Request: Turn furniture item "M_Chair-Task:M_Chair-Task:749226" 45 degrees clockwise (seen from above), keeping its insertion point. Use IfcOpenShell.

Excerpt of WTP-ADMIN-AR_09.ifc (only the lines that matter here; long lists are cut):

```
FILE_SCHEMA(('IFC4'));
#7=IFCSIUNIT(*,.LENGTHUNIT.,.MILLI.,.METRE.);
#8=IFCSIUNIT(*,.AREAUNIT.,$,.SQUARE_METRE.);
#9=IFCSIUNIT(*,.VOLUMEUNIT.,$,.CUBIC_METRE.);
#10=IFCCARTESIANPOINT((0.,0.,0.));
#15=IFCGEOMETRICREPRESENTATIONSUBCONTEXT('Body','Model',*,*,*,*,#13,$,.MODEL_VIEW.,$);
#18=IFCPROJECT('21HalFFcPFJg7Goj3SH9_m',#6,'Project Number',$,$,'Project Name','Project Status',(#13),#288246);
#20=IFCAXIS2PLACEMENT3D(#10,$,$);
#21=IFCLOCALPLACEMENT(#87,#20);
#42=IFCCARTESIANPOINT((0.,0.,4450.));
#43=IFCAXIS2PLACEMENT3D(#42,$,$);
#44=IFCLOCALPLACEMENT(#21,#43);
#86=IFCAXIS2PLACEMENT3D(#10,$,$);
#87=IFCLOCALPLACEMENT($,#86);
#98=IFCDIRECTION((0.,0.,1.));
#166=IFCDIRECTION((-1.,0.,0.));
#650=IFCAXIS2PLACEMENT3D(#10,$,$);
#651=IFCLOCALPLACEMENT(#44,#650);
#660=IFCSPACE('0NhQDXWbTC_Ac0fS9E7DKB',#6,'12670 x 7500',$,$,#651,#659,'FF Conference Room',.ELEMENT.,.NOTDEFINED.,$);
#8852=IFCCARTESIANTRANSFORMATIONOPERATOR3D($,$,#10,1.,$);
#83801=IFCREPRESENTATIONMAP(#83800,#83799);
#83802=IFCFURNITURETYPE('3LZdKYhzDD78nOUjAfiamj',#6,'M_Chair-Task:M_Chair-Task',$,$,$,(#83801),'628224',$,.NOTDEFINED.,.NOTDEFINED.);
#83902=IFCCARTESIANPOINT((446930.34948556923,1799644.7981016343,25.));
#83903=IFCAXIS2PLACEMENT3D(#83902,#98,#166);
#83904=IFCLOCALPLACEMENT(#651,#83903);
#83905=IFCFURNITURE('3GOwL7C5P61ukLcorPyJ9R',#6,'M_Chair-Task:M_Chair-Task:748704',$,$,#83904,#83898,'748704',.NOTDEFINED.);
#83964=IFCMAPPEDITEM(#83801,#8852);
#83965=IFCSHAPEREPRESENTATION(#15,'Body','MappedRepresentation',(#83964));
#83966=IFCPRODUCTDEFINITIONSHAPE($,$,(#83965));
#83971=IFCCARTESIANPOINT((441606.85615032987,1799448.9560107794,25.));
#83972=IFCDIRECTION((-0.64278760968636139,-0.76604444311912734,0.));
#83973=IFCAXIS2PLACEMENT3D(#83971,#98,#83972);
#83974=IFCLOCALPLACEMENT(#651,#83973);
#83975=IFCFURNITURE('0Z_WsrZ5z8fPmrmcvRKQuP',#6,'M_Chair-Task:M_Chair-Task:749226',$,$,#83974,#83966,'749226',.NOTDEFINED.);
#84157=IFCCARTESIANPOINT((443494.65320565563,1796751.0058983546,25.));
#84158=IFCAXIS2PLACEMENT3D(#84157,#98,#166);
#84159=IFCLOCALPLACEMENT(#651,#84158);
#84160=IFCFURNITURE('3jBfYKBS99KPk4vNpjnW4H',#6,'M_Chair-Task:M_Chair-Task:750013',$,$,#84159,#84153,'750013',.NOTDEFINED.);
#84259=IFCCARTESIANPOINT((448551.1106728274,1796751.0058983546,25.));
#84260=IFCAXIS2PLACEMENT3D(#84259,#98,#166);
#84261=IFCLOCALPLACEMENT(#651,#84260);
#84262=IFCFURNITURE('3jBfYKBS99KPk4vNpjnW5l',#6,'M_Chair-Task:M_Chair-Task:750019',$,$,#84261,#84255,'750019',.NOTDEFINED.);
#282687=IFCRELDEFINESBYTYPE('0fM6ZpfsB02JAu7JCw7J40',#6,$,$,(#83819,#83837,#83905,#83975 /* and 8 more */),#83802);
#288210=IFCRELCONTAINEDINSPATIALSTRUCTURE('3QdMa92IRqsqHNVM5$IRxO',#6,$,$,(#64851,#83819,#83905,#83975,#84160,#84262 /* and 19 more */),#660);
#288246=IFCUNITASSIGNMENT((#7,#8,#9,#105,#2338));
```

```python
import ifcopenshell
import ifcopenshell.api.geometry
import ifcopenshell.util.placement

model = ifcopenshell.open("WTP-ADMIN-AR_09.ifc")

item = model.by_guid("0Z_WsrZ5z8fPmrmcvRKQuP")
matrix = ifcopenshell.util.placement.get_local_placement(item.ObjectPlacement)
matrix = matrix @ ifcopenshell.util.placement.rotation(-45, "Z")
ifcopenshell.api.geometry.edit_object_placement(model, product=item, matrix=matrix, is_si=False)

print(ifcopenshell.util.placement.get_local_placement(item.ObjectPlacement).round(3) + 0.0)

model.write("WTP-ADMIN-AR_09_rev.ifc")
```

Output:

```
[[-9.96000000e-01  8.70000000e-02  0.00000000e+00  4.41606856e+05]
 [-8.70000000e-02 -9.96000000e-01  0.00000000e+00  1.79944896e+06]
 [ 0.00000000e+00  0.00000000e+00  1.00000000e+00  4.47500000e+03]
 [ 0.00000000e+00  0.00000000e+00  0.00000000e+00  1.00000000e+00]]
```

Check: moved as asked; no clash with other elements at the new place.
